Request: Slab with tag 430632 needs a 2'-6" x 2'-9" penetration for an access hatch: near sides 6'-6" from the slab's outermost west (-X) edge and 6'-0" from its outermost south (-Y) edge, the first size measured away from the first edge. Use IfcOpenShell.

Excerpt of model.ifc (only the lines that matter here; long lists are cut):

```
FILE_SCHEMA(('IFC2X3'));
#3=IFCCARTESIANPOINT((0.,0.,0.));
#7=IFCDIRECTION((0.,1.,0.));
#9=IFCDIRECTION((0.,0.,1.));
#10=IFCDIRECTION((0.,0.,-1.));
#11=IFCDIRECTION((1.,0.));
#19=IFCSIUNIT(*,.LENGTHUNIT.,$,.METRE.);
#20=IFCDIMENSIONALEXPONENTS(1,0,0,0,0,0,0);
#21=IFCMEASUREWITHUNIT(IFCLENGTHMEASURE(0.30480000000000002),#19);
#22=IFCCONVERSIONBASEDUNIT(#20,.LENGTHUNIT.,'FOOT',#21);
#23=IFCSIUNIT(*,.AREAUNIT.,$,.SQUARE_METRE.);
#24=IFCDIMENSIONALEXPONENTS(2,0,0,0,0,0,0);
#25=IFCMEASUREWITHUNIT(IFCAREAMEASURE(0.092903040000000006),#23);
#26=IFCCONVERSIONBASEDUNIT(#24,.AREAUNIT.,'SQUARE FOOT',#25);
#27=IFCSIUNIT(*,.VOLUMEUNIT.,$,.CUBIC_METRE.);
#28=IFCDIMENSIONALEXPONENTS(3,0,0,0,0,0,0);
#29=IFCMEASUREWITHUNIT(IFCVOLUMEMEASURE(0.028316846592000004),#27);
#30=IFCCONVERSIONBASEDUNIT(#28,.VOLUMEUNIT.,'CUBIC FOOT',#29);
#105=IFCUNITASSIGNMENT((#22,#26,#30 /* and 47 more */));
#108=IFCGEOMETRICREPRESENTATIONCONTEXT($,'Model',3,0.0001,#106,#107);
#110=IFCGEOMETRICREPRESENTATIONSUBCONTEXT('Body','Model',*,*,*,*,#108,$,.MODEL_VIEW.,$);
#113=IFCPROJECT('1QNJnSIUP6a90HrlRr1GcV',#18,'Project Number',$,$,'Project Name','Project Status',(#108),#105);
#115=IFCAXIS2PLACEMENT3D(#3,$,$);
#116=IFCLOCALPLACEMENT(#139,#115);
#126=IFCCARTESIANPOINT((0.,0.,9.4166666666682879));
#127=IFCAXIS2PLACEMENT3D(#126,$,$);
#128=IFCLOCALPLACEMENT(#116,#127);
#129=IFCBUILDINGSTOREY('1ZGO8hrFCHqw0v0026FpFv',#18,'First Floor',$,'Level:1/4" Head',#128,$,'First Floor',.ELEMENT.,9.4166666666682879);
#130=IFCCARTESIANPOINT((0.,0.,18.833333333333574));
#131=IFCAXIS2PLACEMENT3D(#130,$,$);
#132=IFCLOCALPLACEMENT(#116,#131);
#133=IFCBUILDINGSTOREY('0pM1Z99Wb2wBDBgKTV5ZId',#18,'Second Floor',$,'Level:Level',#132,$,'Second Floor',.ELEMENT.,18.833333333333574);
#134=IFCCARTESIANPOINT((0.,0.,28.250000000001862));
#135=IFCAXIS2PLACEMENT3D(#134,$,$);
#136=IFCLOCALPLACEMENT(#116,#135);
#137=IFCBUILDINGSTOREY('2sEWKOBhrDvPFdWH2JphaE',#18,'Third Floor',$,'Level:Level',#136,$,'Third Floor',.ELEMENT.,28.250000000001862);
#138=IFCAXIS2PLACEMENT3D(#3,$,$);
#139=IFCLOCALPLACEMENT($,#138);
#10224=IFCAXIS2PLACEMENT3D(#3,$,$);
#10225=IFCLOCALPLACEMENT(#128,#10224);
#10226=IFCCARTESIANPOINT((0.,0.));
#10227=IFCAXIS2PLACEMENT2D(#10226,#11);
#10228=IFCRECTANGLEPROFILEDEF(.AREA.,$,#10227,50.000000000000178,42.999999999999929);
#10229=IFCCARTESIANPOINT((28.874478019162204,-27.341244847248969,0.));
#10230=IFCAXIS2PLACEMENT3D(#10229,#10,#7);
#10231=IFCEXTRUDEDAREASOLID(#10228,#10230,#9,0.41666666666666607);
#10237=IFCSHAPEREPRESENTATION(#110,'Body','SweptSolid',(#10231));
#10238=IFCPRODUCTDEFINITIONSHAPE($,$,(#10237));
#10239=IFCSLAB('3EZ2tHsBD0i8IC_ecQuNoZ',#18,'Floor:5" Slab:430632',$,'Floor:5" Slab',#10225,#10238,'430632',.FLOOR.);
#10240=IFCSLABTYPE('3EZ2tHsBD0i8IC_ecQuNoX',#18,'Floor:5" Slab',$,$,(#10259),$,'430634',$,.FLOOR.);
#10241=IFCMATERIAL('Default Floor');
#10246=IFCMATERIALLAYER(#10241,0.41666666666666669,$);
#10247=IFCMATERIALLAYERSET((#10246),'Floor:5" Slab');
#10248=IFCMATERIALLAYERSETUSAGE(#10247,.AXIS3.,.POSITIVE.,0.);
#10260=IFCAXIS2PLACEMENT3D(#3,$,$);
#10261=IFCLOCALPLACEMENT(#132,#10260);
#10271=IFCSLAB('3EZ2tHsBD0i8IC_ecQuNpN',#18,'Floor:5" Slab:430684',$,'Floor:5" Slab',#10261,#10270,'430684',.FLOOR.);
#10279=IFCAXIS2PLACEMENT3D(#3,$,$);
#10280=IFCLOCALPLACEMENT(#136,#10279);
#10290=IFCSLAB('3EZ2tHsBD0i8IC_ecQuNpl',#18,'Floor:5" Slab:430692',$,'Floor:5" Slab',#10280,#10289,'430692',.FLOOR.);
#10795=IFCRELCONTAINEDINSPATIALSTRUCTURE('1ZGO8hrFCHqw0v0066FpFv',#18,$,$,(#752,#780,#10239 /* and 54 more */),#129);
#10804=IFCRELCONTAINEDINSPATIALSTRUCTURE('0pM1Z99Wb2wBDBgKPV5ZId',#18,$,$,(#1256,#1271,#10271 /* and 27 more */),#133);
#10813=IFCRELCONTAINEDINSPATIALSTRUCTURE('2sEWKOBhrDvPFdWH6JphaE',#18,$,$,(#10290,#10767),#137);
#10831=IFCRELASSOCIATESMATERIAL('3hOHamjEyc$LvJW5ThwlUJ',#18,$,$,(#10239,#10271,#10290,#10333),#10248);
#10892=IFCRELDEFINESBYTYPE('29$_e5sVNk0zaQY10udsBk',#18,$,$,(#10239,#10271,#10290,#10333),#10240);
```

```python
import numpy as np
import ifcopenshell
import ifcopenshell.api.feature
import ifcopenshell.api.geometry
import ifcopenshell.api.root
import ifcopenshell.geom
import ifcopenshell.util.placement
import ifcopenshell.util.representation
import ifcopenshell.util.shape
import ifcopenshell.util.unit

model = ifcopenshell.open("model.ifc")
unit_scale = ifcopenshell.util.unit.calculate_unit_scale(model)
settings = ifcopenshell.geom.settings()


def volume(element):
    """Net volume in cubic metres, openings subtracted."""
    shape = ifcopenshell.geom.create_shape(settings, element)
    return ifcopenshell.util.shape.get_volume(shape.geometry)


slab = model.by_guid("3EZ2tHsBD0i8IC_ecQuNoZ")
before = volume(slab)

# Extent in the slab's own axes, in metres. The edges named are its -X and -Y sides.
slab_shape = ifcopenshell.geom.create_shape(settings, slab)
vertices = ifcopenshell.util.shape.get_vertices(slab_shape.geometry)
x_min, y_min, bottom = vertices.min(axis=0)
top = vertices[:, 2].max()

opening = ifcopenshell.api.root.create_entity(model, ifc_class="IfcOpeningElement", name="Access hatch opening")
context = ifcopenshell.util.representation.get_context(model, "Model", "Body", "MODEL_VIEW")
width, depth = 0.762, 0.8382
outline = [(0.0, 0.0), (width, 0.0), (width, depth), (0.0, depth), (0.0, 0.0)]
# Overshoot both faces by 50 mm so the cut is clean.
shape = ifcopenshell.api.geometry.add_slab_representation(
    model, context=context, depth=top - bottom + 0.1, polyline=outline
)
ifcopenshell.api.geometry.assign_representation(model, product=opening, representation=shape)

matrix = ifcopenshell.util.placement.get_local_placement(slab.ObjectPlacement)
matrix[:, 3] = matrix @ np.append(np.array([x_min + 1.9812, y_min + 1.8288, bottom - 0.05]) / unit_scale, 1.0)
ifcopenshell.api.geometry.edit_object_placement(model, product=opening, matrix=matrix, is_si=False)
ifcopenshell.api.feature.add_feature(model, feature=opening, element=slab)

after = volume(slab)

print(f"slab volume {before:.3f} -> {after:.3f} m3")

model.write("model_v2.ifc")
```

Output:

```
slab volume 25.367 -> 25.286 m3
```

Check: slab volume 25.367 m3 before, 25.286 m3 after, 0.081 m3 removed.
